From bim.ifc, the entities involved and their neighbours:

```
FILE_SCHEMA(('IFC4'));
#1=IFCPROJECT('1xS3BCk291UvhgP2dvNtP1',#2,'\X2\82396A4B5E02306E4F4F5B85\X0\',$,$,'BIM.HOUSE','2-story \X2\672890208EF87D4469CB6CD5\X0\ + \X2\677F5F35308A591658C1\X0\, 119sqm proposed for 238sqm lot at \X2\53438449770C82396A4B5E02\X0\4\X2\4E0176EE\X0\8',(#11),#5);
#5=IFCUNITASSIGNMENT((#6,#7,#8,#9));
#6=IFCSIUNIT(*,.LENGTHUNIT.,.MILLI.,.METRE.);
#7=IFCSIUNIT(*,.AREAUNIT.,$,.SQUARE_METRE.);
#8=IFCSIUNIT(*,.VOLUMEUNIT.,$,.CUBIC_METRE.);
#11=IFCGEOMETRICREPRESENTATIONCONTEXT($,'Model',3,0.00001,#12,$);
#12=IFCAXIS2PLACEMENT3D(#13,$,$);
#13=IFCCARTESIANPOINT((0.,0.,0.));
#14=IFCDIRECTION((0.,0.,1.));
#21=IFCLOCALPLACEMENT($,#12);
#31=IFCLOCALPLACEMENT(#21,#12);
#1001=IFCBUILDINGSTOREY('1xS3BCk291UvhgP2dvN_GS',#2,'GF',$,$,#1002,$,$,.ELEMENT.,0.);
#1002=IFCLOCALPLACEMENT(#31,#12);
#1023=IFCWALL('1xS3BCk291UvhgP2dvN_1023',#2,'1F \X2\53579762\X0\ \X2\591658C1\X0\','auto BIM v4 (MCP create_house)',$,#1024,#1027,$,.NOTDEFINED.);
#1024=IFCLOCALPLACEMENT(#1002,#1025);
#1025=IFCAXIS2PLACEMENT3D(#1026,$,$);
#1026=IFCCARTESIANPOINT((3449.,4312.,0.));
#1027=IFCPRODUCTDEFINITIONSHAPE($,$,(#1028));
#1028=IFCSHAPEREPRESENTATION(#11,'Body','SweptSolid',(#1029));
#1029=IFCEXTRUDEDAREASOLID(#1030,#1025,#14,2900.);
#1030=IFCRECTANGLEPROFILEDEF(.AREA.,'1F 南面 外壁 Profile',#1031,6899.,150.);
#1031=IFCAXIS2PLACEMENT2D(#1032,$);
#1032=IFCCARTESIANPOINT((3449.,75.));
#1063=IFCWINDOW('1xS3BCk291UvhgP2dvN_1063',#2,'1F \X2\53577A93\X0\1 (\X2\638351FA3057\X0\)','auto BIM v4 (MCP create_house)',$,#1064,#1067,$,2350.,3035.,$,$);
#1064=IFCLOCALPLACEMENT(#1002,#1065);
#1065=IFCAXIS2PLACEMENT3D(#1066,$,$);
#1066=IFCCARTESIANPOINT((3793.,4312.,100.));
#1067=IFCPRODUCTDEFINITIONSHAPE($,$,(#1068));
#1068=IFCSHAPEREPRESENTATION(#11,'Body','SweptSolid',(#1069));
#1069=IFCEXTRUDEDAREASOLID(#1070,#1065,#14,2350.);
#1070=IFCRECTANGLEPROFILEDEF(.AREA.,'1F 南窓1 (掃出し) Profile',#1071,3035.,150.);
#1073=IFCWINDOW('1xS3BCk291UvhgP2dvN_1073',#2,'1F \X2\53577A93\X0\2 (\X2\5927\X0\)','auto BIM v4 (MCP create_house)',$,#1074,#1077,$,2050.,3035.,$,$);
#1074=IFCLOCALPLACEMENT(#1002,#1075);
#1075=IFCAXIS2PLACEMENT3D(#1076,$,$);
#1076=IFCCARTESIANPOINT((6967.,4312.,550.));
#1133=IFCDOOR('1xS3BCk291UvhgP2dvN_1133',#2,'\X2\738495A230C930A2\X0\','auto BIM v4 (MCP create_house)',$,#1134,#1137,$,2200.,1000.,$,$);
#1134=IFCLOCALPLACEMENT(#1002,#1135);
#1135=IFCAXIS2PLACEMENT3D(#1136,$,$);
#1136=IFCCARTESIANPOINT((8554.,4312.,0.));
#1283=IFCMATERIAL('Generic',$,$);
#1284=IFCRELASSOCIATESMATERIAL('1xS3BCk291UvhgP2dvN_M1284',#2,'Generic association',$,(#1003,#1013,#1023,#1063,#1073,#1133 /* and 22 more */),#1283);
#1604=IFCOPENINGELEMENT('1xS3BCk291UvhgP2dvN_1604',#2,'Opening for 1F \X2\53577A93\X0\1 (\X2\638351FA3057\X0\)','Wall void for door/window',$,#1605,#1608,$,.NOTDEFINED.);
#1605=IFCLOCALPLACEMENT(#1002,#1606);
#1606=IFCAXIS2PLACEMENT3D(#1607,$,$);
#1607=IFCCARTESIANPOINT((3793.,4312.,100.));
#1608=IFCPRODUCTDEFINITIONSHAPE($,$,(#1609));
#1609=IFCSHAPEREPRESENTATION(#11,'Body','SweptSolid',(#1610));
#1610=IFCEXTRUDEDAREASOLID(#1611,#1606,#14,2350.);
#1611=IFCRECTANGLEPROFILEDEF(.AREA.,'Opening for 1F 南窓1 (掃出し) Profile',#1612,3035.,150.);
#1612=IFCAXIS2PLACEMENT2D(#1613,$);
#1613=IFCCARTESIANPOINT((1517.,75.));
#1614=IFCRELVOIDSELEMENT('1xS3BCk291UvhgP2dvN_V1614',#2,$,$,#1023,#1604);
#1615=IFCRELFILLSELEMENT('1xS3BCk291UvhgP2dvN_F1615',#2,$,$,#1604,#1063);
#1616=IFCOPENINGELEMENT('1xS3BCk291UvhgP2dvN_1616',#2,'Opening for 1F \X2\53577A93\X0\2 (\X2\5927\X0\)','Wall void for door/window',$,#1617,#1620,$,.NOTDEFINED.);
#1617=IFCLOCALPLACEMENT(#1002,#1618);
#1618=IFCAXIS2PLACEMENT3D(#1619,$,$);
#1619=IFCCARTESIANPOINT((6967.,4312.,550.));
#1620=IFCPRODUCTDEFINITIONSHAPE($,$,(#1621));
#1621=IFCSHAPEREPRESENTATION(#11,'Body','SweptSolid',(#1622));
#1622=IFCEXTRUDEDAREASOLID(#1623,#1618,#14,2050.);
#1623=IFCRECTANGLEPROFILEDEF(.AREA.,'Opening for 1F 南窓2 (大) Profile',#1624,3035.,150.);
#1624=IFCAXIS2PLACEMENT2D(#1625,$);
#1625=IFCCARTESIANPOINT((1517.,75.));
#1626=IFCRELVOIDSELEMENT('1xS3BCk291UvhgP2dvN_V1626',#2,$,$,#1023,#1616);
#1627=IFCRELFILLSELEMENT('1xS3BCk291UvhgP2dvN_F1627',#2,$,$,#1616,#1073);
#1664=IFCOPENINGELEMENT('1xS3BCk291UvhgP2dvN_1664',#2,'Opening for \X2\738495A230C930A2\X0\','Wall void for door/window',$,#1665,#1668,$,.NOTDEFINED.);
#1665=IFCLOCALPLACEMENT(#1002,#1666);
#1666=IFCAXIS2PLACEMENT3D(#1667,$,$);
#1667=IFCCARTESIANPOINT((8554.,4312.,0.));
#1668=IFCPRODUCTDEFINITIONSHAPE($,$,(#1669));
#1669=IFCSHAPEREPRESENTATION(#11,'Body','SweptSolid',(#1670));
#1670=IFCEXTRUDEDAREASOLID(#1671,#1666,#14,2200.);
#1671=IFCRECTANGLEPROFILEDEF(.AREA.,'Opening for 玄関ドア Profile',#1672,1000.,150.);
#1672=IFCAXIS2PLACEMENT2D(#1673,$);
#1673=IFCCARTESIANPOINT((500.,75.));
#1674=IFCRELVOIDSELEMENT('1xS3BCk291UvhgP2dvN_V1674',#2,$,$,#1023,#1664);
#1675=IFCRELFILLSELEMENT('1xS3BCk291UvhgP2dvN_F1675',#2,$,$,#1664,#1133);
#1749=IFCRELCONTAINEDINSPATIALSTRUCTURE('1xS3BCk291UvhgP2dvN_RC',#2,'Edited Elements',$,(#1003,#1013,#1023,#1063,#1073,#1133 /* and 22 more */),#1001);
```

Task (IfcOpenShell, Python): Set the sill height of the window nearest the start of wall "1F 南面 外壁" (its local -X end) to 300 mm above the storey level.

```python
import numpy as np
import ifcopenshell
import ifcopenshell.api.geometry
import ifcopenshell.geom
import ifcopenshell.util.element
import ifcopenshell.util.placement
import ifcopenshell.util.shape
import ifcopenshell.util.unit

model = ifcopenshell.open("bim.ifc")
unit_scale = ifcopenshell.util.unit.calculate_unit_scale(model)

window = model.by_guid("1xS3BCk291UvhgP2dvN_1063")
opening = window.FillsVoids[0].RelatingOpeningElement
storey = ifcopenshell.util.element.get_container(window, ifc_class="IfcBuildingStorey")
level = ifcopenshell.util.placement.get_local_placement(storey.ObjectPlacement)[2, 3]

# The opening's origin need not be at the sill, so measure its lowest point.
shape = ifcopenshell.geom.create_shape(ifcopenshell.geom.settings(), opening)
bottom = ifcopenshell.util.shape.get_shape_bottom_elevation(shape, shape.geometry) / unit_scale
dz = level + 0.3 / unit_scale - bottom

shift = np.array([0.0, 0.0, dz])
# The window is not placed relative to its opening, so move both.
for product in (opening, window):
    matrix = ifcopenshell.util.placement.get_local_placement(product.ObjectPlacement)
    matrix[:3, 3] += shift
    ifcopenshell.api.geometry.edit_object_placement(model, product=product, matrix=matrix, is_si=False)

print(f"moved by {dz * unit_scale:+.3f} m")

model.write("bim_rev.ifc")
```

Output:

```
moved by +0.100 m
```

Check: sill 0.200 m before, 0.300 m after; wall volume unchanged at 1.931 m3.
